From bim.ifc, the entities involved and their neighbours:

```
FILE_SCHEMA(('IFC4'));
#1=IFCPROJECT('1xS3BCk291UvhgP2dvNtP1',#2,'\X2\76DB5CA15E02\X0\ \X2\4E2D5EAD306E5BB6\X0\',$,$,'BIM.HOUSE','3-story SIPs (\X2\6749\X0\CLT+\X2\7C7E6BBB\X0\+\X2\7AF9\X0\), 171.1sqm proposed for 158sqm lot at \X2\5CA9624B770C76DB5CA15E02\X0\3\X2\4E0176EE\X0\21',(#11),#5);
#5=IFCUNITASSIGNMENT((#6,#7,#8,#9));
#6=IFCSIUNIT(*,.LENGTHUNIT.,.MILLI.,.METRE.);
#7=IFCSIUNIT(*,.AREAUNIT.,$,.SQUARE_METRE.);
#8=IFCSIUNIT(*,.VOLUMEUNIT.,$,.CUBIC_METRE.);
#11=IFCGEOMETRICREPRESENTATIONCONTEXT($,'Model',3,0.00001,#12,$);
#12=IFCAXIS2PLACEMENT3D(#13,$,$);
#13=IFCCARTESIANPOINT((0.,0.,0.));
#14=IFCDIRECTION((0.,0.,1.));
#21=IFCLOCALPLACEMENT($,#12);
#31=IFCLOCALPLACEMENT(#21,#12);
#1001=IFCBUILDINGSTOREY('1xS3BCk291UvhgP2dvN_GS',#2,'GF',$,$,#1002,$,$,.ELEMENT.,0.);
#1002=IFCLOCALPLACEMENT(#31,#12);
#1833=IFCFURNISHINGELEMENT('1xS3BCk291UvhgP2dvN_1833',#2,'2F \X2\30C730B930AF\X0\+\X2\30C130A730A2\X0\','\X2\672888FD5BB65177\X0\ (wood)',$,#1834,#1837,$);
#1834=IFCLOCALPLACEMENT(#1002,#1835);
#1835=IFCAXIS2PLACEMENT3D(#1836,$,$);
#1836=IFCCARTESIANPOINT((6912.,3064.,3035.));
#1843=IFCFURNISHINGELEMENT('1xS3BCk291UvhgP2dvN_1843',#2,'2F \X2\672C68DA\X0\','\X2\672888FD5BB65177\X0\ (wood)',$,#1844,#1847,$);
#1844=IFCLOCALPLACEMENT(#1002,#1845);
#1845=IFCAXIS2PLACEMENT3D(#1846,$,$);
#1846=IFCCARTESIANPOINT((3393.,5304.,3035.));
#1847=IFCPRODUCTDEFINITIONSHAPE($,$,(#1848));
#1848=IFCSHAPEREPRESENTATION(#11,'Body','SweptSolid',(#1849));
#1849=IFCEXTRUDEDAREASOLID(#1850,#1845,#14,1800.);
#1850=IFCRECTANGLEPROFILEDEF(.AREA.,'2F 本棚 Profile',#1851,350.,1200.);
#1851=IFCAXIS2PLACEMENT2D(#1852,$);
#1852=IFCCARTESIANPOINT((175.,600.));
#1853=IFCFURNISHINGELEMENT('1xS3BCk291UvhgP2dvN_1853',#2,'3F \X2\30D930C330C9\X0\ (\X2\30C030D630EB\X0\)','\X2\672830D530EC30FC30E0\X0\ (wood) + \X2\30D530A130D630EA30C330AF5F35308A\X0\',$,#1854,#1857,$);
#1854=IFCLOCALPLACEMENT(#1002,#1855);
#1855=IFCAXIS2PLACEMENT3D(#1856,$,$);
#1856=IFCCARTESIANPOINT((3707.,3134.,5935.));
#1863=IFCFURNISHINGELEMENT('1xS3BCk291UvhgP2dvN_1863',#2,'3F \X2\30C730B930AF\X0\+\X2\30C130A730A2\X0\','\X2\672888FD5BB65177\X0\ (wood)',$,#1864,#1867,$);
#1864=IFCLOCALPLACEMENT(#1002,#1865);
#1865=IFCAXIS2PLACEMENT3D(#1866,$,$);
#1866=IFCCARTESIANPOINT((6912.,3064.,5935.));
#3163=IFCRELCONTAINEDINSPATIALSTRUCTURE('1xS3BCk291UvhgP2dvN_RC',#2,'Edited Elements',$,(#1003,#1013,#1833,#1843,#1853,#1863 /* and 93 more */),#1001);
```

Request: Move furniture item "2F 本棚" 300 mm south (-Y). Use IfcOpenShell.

```python
import ifcopenshell
import ifcopenshell.api.geometry
import ifcopenshell.util.placement

model = ifcopenshell.open("bim.ifc")

item = model.by_guid("1xS3BCk291UvhgP2dvN_1843")
matrix = ifcopenshell.util.placement.get_local_placement(item.ObjectPlacement)
matrix[1, 3] -= 300.0
ifcopenshell.api.geometry.edit_object_placement(model, product=item, matrix=matrix, is_si=False)

print(ifcopenshell.util.placement.get_local_placement(item.ObjectPlacement).round(3) + 0.0)

model.write("bim_rev.ifc")
```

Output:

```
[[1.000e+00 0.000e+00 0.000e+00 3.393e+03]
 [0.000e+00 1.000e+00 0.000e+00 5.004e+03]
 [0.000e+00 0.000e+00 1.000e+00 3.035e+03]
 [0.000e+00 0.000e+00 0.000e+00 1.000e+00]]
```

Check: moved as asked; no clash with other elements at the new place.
